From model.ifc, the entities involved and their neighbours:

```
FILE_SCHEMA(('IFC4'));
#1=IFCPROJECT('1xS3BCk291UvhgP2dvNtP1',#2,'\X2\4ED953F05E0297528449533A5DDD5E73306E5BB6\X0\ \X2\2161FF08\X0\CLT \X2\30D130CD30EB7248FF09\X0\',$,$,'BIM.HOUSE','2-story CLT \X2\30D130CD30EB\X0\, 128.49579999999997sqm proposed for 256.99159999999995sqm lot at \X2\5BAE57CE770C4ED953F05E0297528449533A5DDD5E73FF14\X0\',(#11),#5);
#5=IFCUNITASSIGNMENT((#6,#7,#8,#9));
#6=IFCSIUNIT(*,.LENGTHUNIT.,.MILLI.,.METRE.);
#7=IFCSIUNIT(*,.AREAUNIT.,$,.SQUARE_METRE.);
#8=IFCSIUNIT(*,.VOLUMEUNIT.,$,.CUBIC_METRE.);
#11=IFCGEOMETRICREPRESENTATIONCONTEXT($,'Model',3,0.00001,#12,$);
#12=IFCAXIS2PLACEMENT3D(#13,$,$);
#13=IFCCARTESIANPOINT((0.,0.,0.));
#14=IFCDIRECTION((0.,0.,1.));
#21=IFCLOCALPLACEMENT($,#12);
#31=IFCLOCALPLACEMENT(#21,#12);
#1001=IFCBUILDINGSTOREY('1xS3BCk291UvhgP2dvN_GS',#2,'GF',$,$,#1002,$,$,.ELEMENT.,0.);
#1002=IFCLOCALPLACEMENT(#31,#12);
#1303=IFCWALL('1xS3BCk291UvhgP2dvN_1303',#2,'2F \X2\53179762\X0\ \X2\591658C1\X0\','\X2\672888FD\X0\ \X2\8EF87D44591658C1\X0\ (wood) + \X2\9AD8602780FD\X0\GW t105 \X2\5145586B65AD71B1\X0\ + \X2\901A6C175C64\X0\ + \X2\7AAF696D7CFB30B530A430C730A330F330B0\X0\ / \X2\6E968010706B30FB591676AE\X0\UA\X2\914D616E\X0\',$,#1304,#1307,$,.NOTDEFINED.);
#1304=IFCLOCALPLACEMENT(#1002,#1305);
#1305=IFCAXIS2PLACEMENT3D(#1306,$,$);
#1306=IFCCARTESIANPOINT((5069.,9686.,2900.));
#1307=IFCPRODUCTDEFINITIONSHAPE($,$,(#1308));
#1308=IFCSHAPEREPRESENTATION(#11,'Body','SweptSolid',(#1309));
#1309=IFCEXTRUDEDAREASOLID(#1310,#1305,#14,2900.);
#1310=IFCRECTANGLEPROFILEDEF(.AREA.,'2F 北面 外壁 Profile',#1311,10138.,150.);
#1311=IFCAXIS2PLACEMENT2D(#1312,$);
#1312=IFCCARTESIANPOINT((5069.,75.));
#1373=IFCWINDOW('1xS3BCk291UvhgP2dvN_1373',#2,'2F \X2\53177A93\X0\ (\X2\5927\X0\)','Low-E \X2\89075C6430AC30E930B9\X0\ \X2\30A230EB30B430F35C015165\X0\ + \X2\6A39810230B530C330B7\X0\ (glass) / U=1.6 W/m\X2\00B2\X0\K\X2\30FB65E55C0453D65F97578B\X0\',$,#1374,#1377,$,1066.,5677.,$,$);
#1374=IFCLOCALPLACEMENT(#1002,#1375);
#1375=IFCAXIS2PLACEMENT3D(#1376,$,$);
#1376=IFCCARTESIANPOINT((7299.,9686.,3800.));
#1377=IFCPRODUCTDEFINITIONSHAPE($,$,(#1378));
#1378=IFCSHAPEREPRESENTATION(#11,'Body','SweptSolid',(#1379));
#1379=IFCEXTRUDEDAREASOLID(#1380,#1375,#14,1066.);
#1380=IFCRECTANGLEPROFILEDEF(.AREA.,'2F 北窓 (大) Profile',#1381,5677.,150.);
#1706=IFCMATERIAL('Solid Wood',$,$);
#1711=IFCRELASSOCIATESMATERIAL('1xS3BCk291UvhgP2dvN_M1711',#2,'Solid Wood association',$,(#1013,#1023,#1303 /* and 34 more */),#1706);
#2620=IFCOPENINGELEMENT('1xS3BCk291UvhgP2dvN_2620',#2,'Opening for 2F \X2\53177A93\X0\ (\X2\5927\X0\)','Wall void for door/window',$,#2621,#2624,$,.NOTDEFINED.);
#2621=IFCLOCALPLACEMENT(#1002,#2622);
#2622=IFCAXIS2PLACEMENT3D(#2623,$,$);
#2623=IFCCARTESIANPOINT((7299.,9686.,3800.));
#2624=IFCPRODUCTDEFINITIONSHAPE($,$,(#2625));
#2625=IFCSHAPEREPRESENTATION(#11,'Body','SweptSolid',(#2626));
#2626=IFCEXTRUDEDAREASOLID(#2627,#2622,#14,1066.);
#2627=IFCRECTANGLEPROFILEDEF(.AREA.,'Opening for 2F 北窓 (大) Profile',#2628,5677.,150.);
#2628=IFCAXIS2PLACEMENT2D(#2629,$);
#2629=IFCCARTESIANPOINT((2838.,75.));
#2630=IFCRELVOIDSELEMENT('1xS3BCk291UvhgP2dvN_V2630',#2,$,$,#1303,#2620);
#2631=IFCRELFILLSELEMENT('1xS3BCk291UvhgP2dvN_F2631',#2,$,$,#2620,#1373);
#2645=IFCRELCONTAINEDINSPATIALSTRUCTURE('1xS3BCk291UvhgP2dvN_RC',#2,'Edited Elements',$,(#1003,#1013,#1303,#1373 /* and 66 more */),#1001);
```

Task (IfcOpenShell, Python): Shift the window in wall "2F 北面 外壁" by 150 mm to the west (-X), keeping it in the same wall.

```python
import ifcopenshell
import ifcopenshell.api.geometry
import ifcopenshell.util.placement

model = ifcopenshell.open("model.ifc")

window = model.by_guid("1xS3BCk291UvhgP2dvN_1373")
opening = window.FillsVoids[0].RelatingOpeningElement
wall = opening.VoidsElements[0].RelatingBuildingElement

wall_matrix = ifcopenshell.util.placement.get_local_placement(wall.ObjectPlacement)
shift = wall_matrix[:3, 0] * -150.0
before = ifcopenshell.util.placement.get_local_placement(window.ObjectPlacement)[:3, 3].copy()

# The window is not placed relative to its opening, so move both.
for product in (opening, window):
    matrix = ifcopenshell.util.placement.get_local_placement(product.ObjectPlacement)
    matrix[:3, 3] += shift
    ifcopenshell.api.geometry.edit_object_placement(model, product=product, matrix=matrix, is_si=False)

after = ifcopenshell.util.placement.get_local_placement(window.ObjectPlacement)[:3, 3]
print("window moved by", (after - before).round(3) + 0.0)

model.write("model_rev.ifc")
```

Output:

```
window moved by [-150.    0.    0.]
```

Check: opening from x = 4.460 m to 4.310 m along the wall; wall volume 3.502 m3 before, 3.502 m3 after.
